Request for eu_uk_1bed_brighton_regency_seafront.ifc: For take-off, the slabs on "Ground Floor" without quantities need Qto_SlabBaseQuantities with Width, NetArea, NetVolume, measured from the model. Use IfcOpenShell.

First a look at what the model holds.

```python
import ifcopenshell
import ifcopenshell.util.element
import ifcopenshell.util.unit

model = ifcopenshell.open("eu_uk_1bed_brighton_regency_seafront.ifc")
print(model.schema)
for unit_type in ("LENGTHUNIT", "AREAUNIT", "VOLUMEUNIT"):
    print(unit_type, ifcopenshell.util.unit.calculate_unit_scale(model, unit_type))
storey = next(s for s in model.by_type("IfcBuildingStorey") if s.Name == "Ground Floor")
slabs = [e for e in ifcopenshell.util.element.get_decomposition(storey) if e.is_a("IfcSlab")]
for e in sorted(slabs, key=lambda e: e.id()):
    print(e.id(), e.is_a(), e.Name, list(ifcopenshell.util.element.get_psets(e, qtos_only=True)), sep=" | ")
```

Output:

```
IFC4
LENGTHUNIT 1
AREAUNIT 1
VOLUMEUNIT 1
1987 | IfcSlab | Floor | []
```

```python
import ifcopenshell
import ifcopenshell.api.pset
import ifcopenshell.geom
import ifcopenshell.util.element
import ifcopenshell.util.shape
import ifcopenshell.util.unit

model = ifcopenshell.open("eu_uk_1bed_brighton_regency_seafront.ifc")
unit_scale = ifcopenshell.util.unit.calculate_unit_scale(model)
area_scale = ifcopenshell.util.unit.calculate_unit_scale(model, "AREAUNIT")
volume_scale = ifcopenshell.util.unit.calculate_unit_scale(model, "VOLUMEUNIT")
settings = ifcopenshell.geom.settings()

storey = next(s for s in model.by_type("IfcBuildingStorey") if s.Name == "Ground Floor")
slabs = [e for e in ifcopenshell.util.element.get_decomposition(storey) if e.is_a("IfcSlab")]

for e in sorted(slabs, key=lambda e: e.id()):
    if ifcopenshell.util.element.get_psets(e, qtos_only=True, should_inherit=False):
        continue
    # Geometry comes back in metres, in the element's own axes.
    shape = ifcopenshell.geom.create_shape(settings, e)
    values = {
        "Width": ifcopenshell.util.shape.get_z(shape.geometry) / unit_scale,
        "NetArea": ifcopenshell.util.shape.get_footprint_area(shape.geometry) / area_scale,
        "NetVolume": ifcopenshell.util.shape.get_volume(shape.geometry) / volume_scale,
    }
    qto = ifcopenshell.api.pset.add_qto(model, product=e, name="Qto_SlabBaseQuantities")
    ifcopenshell.api.pset.edit_qto(model, qto=qto, properties=values)
    print(e.id(), {k: round(v, 3) for k, v in values.items()})

model.write("eu_uk_1bed_brighton_regency_seafront_updated.ifc")
```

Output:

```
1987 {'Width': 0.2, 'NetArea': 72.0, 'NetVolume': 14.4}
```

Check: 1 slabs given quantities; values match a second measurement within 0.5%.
